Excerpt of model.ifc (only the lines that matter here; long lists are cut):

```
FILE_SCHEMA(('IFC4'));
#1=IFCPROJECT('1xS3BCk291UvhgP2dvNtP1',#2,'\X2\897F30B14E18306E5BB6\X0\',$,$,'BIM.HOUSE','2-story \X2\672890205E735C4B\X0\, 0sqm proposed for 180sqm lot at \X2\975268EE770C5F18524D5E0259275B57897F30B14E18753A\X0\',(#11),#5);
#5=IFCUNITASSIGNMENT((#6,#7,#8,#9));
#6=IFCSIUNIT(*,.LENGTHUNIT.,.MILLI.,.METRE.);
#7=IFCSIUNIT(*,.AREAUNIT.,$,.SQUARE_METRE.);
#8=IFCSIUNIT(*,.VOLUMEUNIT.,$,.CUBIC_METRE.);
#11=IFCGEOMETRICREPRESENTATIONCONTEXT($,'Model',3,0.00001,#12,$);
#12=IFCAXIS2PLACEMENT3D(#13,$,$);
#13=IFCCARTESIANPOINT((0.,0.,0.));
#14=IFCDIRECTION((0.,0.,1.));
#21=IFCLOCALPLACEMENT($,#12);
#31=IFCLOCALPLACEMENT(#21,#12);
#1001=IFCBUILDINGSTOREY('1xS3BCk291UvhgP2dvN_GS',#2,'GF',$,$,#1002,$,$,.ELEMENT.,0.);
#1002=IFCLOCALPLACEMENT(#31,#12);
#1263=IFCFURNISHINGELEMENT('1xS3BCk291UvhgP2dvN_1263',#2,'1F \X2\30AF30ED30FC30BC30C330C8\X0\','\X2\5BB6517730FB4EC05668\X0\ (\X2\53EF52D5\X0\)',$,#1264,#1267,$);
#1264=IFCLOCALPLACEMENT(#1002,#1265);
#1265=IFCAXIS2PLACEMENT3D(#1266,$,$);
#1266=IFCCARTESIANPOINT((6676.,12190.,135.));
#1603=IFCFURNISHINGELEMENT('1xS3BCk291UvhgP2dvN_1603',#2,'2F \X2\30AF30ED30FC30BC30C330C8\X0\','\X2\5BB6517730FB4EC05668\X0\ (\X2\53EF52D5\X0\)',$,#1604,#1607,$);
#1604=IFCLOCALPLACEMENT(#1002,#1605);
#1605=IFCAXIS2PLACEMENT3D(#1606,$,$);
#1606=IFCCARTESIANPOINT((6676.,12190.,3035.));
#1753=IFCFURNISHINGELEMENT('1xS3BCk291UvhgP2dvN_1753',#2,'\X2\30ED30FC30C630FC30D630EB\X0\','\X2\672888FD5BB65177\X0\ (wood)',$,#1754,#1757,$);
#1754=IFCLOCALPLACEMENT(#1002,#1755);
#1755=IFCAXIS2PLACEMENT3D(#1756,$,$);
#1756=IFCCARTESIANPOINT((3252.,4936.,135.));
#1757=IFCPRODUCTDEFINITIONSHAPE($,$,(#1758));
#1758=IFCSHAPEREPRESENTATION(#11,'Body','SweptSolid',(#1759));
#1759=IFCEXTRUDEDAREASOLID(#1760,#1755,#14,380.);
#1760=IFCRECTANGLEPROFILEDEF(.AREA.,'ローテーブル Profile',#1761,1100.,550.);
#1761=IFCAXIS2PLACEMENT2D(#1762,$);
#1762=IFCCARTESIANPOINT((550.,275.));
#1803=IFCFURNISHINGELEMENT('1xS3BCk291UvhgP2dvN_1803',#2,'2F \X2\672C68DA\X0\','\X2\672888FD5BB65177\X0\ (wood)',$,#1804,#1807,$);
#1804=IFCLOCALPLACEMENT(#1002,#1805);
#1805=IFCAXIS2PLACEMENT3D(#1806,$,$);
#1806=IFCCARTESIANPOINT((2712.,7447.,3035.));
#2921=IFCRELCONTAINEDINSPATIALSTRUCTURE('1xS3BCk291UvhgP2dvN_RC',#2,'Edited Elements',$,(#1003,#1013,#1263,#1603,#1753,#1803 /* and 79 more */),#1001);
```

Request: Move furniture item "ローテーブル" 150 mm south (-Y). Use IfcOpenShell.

```python
import ifcopenshell
import ifcopenshell.api.geometry
import ifcopenshell.util.placement

model = ifcopenshell.open("model.ifc")

item = model.by_guid("1xS3BCk291UvhgP2dvN_1753")
matrix = ifcopenshell.util.placement.get_local_placement(item.ObjectPlacement)
matrix[1, 3] -= 150.0
ifcopenshell.api.geometry.edit_object_placement(model, product=item, matrix=matrix, is_si=False)

print(ifcopenshell.util.placement.get_local_placement(item.ObjectPlacement).round(3) + 0.0)

model.write("model_edited.ifc")
```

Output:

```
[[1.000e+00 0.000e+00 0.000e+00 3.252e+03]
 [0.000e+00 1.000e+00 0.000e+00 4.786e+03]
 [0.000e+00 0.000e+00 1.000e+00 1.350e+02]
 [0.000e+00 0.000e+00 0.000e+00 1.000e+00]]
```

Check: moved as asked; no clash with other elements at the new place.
